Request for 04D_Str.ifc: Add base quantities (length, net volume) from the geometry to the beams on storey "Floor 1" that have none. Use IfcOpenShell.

First a look at what the model holds.

```python
import ifcopenshell
import ifcopenshell.util.element
import ifcopenshell.util.unit

model = ifcopenshell.open("04D_Str.ifc")
print(model.schema)
for unit_type in ("LENGTHUNIT", "AREAUNIT", "VOLUMEUNIT"):
    print(unit_type, ifcopenshell.util.unit.calculate_unit_scale(model, unit_type))
storey = next(s for s in model.by_type("IfcBuildingStorey") if s.Name == "Floor 1")
beams = [e for e in ifcopenshell.util.element.get_decomposition(storey) if e.is_a("IfcBeam")]
for e in sorted(beams, key=lambda e: e.id()):
    print(e.id(), e.is_a(), e.Name, list(ifcopenshell.util.element.get_psets(e, qtos_only=True)), sep=" | ")
```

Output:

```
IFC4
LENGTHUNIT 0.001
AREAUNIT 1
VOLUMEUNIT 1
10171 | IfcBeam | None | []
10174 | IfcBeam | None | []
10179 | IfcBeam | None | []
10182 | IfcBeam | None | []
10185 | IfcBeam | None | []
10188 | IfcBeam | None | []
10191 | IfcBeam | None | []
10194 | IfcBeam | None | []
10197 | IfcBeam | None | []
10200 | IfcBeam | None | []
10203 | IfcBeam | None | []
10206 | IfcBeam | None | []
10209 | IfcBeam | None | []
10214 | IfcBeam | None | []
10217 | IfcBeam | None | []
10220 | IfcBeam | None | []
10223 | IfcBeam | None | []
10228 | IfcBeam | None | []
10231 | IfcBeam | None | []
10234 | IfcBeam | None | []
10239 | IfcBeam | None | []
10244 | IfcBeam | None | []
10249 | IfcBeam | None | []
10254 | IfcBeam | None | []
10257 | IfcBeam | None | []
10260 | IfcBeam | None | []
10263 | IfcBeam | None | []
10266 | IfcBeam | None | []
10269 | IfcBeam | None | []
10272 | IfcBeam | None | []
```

```python
import ifcopenshell
import ifcopenshell.api.pset
import ifcopenshell.geom
import ifcopenshell.util.element
import ifcopenshell.util.shape
import ifcopenshell.util.unit

model = ifcopenshell.open("04D_Str.ifc")
unit_scale = ifcopenshell.util.unit.calculate_unit_scale(model)
volume_scale = ifcopenshell.util.unit.calculate_unit_scale(model, "VOLUMEUNIT")
settings = ifcopenshell.geom.settings()

storey = next(s for s in model.by_type("IfcBuildingStorey") if s.Name == "Floor 1")
beams = [e for e in ifcopenshell.util.element.get_decomposition(storey) if e.is_a("IfcBeam")]

for e in sorted(beams, key=lambda e: e.id()):
    if ifcopenshell.util.element.get_psets(e, qtos_only=True, should_inherit=False):
        continue
    # Geometry comes back in metres, in the element's own axes.
    shape = ifcopenshell.geom.create_shape(settings, e)
    values = {
        "Length": ifcopenshell.util.shape.get_max_xyz(shape.geometry) / unit_scale,
        "NetVolume": ifcopenshell.util.shape.get_volume(shape.geometry) / volume_scale,
    }
    qto = ifcopenshell.api.pset.add_qto(model, product=e, name="Qto_BeamBaseQuantities")
    ifcopenshell.api.pset.edit_qto(model, qto=qto, properties=values)
    print(e.id(), {k: round(v, 3) for k, v in values.items()})

model.write("04D_Str_rev.ifc")
```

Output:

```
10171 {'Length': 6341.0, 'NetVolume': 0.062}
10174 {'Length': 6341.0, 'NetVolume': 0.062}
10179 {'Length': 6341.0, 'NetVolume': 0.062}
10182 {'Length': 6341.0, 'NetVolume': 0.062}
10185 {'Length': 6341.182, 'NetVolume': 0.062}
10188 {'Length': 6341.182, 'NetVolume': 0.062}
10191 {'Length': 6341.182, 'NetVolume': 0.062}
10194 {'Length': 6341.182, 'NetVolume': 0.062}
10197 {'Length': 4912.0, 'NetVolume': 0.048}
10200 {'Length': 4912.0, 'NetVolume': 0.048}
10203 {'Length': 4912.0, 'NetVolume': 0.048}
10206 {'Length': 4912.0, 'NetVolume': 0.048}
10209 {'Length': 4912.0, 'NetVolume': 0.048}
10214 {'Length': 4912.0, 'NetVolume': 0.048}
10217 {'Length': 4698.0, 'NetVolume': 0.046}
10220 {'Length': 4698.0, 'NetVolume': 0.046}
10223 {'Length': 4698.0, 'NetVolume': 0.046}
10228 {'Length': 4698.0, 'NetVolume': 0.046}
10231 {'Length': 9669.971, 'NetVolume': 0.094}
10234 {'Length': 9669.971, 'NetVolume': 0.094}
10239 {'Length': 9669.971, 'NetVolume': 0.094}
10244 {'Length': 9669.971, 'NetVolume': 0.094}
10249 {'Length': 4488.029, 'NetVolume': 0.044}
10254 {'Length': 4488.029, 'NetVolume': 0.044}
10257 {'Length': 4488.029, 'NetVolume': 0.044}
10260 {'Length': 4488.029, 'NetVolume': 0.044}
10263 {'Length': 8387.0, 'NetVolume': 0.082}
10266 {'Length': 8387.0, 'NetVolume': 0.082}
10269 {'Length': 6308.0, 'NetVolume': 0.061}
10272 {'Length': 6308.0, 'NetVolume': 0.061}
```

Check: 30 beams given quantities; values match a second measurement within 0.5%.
